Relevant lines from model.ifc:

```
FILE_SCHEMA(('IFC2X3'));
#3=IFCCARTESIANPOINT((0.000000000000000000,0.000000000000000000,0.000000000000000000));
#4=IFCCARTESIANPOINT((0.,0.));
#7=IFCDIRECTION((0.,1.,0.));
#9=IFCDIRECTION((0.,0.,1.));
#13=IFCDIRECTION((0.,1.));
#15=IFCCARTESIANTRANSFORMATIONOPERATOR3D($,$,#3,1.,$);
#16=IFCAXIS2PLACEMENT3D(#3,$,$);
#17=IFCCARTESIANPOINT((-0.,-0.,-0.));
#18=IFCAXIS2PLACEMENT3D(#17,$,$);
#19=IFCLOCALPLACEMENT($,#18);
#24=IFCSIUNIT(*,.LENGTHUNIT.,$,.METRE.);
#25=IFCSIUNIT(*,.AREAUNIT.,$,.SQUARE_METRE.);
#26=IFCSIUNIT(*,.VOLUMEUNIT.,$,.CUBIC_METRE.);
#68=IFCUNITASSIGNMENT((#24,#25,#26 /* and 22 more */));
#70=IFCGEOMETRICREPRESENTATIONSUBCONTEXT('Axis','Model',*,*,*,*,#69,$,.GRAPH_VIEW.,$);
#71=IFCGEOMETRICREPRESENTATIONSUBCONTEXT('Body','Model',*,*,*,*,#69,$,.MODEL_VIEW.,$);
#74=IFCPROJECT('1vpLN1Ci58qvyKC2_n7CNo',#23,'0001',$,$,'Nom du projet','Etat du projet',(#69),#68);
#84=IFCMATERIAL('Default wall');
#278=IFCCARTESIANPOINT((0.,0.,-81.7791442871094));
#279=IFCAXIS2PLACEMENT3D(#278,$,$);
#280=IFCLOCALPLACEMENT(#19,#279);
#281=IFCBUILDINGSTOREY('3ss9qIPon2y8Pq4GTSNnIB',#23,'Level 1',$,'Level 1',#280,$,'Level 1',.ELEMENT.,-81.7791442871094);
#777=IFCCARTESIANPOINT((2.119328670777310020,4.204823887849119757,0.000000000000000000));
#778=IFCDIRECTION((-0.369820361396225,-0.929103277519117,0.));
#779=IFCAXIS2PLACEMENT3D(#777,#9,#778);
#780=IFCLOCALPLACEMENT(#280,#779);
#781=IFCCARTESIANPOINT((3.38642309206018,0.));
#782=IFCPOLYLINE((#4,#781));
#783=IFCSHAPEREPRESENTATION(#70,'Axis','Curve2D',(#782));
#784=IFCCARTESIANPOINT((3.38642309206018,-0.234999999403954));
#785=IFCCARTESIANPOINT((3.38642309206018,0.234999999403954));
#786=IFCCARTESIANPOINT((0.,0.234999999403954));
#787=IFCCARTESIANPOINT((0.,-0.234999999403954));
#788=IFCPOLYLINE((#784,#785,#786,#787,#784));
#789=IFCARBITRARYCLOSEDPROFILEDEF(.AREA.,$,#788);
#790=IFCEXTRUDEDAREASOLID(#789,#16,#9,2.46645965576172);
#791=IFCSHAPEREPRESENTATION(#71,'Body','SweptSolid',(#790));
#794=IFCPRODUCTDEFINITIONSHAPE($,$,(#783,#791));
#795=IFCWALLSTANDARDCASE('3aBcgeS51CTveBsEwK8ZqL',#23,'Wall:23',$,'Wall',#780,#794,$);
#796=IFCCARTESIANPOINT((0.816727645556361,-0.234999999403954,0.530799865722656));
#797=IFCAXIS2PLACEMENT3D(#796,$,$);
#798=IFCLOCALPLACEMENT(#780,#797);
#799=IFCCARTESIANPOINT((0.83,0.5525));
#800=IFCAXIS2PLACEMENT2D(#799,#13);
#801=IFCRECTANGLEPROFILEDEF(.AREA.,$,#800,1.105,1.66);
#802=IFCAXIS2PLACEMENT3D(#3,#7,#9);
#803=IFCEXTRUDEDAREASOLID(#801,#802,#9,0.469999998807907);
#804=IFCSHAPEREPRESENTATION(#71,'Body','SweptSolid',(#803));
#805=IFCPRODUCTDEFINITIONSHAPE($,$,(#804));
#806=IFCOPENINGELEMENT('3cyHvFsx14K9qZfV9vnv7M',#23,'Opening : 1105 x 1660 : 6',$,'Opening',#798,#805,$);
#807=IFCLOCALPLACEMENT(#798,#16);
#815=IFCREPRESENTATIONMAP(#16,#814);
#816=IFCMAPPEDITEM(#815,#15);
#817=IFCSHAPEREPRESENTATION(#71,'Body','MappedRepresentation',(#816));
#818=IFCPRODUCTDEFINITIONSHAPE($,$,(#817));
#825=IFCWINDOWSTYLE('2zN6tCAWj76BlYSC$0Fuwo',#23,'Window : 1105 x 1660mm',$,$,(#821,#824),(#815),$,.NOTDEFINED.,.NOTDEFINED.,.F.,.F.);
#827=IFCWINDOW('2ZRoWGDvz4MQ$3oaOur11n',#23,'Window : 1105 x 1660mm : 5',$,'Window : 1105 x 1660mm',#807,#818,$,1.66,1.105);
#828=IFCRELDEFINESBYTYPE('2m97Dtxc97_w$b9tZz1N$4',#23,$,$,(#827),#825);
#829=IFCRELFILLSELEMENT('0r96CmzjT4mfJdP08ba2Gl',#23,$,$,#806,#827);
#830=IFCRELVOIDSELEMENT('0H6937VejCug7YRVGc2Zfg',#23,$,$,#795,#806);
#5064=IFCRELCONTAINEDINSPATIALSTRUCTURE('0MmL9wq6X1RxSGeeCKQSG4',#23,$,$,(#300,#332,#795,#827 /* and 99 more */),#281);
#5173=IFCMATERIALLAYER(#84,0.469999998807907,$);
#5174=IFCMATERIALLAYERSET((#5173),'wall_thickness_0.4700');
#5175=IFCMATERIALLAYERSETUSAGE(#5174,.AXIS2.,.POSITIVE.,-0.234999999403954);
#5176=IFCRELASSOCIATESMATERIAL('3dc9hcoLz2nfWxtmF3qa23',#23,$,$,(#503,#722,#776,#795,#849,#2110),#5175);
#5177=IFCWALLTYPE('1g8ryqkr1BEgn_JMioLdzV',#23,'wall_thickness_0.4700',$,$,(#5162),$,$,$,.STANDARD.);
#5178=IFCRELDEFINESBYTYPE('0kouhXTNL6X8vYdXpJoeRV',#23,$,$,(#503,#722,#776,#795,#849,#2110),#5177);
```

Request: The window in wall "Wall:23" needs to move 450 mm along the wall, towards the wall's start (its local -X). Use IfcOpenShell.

```python
import ifcopenshell
import ifcopenshell.api.geometry
import ifcopenshell.util.placement
import ifcopenshell.util.unit

model = ifcopenshell.open("model.ifc")
unit_scale = ifcopenshell.util.unit.calculate_unit_scale(model)

window = model.by_guid("2ZRoWGDvz4MQ$3oaOur11n")
opening = window.FillsVoids[0].RelatingOpeningElement
wall = opening.VoidsElements[0].RelatingBuildingElement

wall_matrix = ifcopenshell.util.placement.get_local_placement(wall.ObjectPlacement)
shift = wall_matrix[:3, 0] * -0.45 / unit_scale
before = ifcopenshell.util.placement.get_local_placement(window.ObjectPlacement)[:3, 3].copy()

# The window is placed relative to its opening, so it follows when the opening moves.
matrix = ifcopenshell.util.placement.get_local_placement(opening.ObjectPlacement)
matrix[:3, 3] += shift
ifcopenshell.api.geometry.edit_object_placement(
    model, product=opening, matrix=matrix, is_si=False, should_transform_children=True
)

after = ifcopenshell.util.placement.get_local_placement(window.ObjectPlacement)[:3, 3]
print("window moved by", (after - before).round(3) + 0.0)

model.write("model_edited.ifc")
```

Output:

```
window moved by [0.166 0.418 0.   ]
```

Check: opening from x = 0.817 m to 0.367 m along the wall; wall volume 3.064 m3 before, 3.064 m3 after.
